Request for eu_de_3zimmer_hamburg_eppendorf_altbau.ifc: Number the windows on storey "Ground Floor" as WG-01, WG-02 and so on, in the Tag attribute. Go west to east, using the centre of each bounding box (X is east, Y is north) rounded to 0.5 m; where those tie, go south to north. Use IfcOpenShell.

First a look at what the model holds.

```python
import ifcopenshell
import ifcopenshell.util.element
import ifcopenshell.util.placement

model = ifcopenshell.open("eu_de_3zimmer_hamburg_eppendorf_altbau.ifc")
print(model.schema)
storey = next(s for s in model.by_type("IfcBuildingStorey") if s.Name == "Ground Floor")
windows = [e for e in ifcopenshell.util.element.get_decomposition(storey) if e.is_a("IfcWindow")]
for e in sorted(windows, key=lambda e: e.id()):
    origin = ifcopenshell.util.placement.get_local_placement(e.ObjectPlacement)[:3, 3]
    print(e.id(), e.Tag, e.Name, origin.round(2) + 0.0, sep=" | ")
```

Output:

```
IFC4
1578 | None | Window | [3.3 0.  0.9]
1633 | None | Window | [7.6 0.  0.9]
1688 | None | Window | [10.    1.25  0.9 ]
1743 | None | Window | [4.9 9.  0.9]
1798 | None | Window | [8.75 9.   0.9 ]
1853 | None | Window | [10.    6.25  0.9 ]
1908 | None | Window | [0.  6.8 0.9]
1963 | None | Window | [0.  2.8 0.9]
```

```python
import ifcopenshell
import ifcopenshell.geom
import ifcopenshell.util.element
import ifcopenshell.util.shape

model = ifcopenshell.open("eu_de_3zimmer_hamburg_eppendorf_altbau.ifc")
settings = ifcopenshell.geom.settings()
settings.set("use-world-coords", True)


def centre(element):
    shape = ifcopenshell.geom.create_shape(settings, element)
    return ifcopenshell.util.shape.get_bbox_centroid(shape.geometry)


storey = next(s for s in model.by_type("IfcBuildingStorey") if s.Name == "Ground Floor")
windows = [e for e in ifcopenshell.util.element.get_decomposition(storey) if e.is_a("IfcWindow")]

# Insertion points can sit at a corner or the storey origin, so sort by the geometry (in metres).
centres = {e: centre(e) for e in windows}
windows.sort(key=lambda e: (round(centres[e][0] / 0.5), centres[e][1]))

for i, e in enumerate(windows, start=1):
    number = f"WG-{i:02d}"
    e.Tag = number
    print(e.id(), number)

model.write("eu_de_3zimmer_hamburg_eppendorf_altbau-out.ifc")
```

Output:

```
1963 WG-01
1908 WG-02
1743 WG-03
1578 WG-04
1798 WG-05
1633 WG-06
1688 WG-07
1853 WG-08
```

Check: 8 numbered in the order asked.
